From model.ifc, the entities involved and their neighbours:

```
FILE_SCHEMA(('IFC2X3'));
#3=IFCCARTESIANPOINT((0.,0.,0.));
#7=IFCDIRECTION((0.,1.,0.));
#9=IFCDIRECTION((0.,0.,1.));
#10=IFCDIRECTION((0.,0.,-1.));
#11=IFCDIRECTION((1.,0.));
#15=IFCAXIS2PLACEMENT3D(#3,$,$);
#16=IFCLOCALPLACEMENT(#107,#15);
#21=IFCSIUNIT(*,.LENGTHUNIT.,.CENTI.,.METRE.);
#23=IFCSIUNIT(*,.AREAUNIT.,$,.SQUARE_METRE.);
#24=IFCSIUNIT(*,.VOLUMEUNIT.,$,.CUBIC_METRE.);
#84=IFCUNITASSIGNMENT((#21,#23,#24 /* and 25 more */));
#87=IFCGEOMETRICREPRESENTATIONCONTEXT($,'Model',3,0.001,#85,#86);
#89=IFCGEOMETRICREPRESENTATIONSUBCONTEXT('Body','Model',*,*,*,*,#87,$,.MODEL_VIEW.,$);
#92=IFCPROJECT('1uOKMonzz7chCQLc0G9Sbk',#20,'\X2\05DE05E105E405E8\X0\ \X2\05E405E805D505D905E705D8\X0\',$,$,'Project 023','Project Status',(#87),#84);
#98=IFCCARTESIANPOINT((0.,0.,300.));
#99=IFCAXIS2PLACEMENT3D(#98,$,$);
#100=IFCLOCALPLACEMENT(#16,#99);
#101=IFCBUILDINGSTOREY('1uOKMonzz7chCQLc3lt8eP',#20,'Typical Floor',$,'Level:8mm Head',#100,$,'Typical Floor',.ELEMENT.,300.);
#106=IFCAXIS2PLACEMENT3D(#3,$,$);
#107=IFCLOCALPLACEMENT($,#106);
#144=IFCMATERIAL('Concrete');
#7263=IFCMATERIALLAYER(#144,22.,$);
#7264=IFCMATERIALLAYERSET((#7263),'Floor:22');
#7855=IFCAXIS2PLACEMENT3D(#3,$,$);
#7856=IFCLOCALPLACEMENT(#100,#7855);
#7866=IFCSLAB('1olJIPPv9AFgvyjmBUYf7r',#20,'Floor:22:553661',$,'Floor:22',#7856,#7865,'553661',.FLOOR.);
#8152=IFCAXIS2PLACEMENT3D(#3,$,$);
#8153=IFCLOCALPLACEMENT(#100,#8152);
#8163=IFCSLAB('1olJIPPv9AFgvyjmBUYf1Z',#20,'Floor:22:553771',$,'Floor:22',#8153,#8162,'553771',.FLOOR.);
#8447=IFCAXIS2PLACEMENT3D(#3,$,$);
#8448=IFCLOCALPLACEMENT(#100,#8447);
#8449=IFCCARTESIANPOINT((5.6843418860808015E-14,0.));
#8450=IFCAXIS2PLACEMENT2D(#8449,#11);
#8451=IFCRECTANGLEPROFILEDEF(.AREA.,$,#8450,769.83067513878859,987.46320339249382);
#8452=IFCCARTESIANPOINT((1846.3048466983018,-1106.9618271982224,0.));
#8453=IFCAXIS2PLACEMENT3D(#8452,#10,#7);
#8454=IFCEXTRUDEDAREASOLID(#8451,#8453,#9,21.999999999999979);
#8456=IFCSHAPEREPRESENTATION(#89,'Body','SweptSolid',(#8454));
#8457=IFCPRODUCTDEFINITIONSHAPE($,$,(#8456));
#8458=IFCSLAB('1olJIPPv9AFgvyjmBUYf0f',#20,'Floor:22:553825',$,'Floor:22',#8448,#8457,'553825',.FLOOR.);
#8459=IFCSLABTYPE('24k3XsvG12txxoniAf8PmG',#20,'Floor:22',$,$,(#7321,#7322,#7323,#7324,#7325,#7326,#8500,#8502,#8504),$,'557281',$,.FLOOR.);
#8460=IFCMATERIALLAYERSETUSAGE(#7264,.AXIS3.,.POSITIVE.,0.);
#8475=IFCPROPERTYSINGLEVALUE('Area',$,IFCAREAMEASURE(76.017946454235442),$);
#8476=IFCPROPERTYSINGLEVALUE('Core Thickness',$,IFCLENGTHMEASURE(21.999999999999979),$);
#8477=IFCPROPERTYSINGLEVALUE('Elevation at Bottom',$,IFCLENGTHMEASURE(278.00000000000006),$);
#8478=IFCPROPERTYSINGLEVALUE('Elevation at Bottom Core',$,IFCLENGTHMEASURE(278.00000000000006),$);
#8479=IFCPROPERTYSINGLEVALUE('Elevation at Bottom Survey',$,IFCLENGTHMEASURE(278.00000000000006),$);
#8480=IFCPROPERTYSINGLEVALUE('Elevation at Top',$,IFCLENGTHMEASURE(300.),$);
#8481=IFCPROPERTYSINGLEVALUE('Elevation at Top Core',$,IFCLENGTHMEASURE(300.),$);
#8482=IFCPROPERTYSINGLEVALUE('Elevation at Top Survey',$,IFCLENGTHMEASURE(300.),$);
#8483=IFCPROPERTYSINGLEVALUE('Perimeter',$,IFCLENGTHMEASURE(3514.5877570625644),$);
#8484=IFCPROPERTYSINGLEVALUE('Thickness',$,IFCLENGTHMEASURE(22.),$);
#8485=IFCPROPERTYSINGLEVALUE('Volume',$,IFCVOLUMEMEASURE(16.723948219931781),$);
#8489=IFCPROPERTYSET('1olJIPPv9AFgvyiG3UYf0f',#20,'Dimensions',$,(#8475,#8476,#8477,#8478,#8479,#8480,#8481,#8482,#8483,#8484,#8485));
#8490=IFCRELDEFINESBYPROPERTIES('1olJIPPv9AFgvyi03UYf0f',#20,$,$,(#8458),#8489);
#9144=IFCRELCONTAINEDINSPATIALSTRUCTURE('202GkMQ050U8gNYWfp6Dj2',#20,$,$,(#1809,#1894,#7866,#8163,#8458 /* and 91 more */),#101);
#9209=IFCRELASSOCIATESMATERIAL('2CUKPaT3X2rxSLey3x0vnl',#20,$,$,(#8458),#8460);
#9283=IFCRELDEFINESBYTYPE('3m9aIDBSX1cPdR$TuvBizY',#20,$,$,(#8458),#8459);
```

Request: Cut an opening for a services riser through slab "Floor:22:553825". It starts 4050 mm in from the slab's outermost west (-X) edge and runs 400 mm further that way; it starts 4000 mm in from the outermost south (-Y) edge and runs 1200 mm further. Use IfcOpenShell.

```python
import numpy as np
import ifcopenshell
import ifcopenshell.api.feature
import ifcopenshell.api.geometry
import ifcopenshell.api.pset
import ifcopenshell.api.root
import ifcopenshell.geom
import ifcopenshell.util.element
import ifcopenshell.util.placement
import ifcopenshell.util.representation
import ifcopenshell.util.shape
import ifcopenshell.util.unit

model = ifcopenshell.open("model.ifc")
unit_scale = ifcopenshell.util.unit.calculate_unit_scale(model)
area_scale = ifcopenshell.util.unit.calculate_unit_scale(model, "AREAUNIT")
volume_scale = ifcopenshell.util.unit.calculate_unit_scale(model, "VOLUMEUNIT")
settings = ifcopenshell.geom.settings()


def volume(element):
    """Net volume in cubic metres, openings subtracted."""
    shape = ifcopenshell.geom.create_shape(settings, element)
    return ifcopenshell.util.shape.get_volume(shape.geometry)


slab = model.by_guid("1olJIPPv9AFgvyjmBUYf0f")
before = volume(slab)

# Extent in the slab's own axes, in metres. The edges named are its -X and -Y sides.
slab_shape = ifcopenshell.geom.create_shape(settings, slab)
vertices = ifcopenshell.util.shape.get_vertices(slab_shape.geometry)
x_min, y_min, bottom = vertices.min(axis=0)
top = vertices[:, 2].max()

opening = ifcopenshell.api.root.create_entity(model, ifc_class="IfcOpeningElement", name="Services riser opening")
context = ifcopenshell.util.representation.get_context(model, "Model", "Body", "MODEL_VIEW")
width, depth = 0.4, 1.2
outline = [(0.0, 0.0), (width, 0.0), (width, depth), (0.0, depth), (0.0, 0.0)]
# Overshoot both faces by 50 mm so the cut is clean.
shape = ifcopenshell.api.geometry.add_slab_representation(
    model, context=context, depth=top - bottom + 0.1, polyline=outline
)
ifcopenshell.api.geometry.assign_representation(model, product=opening, representation=shape)

matrix = ifcopenshell.util.placement.get_local_placement(slab.ObjectPlacement)
matrix[:, 3] = matrix @ np.append(np.array([x_min + 4.05, y_min + 4, bottom - 0.05]) / unit_scale, 1.0)
ifcopenshell.api.geometry.edit_object_placement(model, product=opening, matrix=matrix, is_si=False)
ifcopenshell.api.feature.add_feature(model, feature=opening, element=slab)

after = volume(slab)

# Update the slab's stored quantities.
pset = model.by_id(ifcopenshell.util.element.get_pset(slab, "Dimensions", should_inherit=False)["id"])
ifcopenshell.api.pset.edit_pset(model, pset=pset, properties={
    "Area": model.create_entity("IfcAreaMeasure", after / (top - bottom) / area_scale),
    "Volume": model.create_entity("IfcVolumeMeasure", after / volume_scale),
})

print(f"slab volume {before:.3f} -> {after:.3f} m3")

model.write("model_updated.ifc")
```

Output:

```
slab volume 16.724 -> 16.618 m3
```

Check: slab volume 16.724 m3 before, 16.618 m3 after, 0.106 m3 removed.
